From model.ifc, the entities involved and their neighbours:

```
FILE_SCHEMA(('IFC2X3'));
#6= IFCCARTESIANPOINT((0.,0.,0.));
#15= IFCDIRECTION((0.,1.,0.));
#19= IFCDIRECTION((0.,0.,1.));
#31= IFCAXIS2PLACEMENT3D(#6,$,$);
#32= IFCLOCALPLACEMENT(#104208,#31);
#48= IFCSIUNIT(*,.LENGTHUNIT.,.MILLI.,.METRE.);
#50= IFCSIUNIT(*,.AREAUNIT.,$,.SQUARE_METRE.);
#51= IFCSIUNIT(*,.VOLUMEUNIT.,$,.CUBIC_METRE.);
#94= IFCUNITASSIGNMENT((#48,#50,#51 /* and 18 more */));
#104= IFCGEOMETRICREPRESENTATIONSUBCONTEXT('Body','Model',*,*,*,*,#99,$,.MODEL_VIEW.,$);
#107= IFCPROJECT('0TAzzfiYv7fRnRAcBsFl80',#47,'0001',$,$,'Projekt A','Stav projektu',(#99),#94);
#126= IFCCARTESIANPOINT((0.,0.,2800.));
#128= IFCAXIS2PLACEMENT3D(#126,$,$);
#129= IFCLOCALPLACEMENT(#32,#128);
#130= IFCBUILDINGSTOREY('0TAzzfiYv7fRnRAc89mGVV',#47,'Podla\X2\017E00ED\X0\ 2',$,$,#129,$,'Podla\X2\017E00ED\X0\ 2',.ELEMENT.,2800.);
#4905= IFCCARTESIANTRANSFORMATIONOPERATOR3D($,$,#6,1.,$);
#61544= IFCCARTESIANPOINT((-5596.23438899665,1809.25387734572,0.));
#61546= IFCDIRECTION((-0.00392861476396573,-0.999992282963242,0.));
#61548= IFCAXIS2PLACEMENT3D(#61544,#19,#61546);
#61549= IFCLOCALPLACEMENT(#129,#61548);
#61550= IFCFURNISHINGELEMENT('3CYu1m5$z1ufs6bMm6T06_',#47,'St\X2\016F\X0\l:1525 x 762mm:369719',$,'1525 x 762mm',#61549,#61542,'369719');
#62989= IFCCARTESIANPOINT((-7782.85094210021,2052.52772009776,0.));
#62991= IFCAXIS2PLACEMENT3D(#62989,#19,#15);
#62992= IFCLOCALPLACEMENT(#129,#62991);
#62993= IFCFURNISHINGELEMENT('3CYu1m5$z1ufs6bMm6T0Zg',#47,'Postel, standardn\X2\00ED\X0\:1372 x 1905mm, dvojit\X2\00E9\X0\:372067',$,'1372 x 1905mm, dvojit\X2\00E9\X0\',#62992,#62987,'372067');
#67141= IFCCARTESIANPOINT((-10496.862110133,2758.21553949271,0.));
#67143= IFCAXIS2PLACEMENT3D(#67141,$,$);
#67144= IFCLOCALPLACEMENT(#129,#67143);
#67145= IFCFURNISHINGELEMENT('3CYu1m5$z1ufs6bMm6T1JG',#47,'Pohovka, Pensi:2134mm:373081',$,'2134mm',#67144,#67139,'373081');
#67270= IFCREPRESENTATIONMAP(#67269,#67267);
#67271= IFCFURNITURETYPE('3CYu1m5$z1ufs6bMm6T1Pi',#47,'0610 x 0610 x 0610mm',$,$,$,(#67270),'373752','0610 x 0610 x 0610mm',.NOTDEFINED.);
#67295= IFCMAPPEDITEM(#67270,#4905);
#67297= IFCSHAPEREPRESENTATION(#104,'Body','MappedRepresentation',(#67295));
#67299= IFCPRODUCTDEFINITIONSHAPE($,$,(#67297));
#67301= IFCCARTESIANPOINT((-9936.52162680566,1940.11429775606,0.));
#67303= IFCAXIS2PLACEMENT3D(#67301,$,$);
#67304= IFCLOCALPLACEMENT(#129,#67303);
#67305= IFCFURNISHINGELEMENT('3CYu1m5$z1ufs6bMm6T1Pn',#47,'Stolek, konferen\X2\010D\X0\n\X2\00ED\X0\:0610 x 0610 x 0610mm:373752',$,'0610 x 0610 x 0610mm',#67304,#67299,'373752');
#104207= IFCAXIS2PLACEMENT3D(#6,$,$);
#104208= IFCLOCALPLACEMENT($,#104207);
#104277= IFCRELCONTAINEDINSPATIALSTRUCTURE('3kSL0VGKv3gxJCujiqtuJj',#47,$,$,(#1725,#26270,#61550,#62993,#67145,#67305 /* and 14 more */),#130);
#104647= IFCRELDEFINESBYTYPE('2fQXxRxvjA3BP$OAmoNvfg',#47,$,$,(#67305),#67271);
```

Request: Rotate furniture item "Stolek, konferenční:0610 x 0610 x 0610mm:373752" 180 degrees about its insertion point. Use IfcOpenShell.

```python
import ifcopenshell
import ifcopenshell.api.geometry
import ifcopenshell.util.placement

model = ifcopenshell.open("model.ifc")

item = model.by_id(67305)
matrix = ifcopenshell.util.placement.get_local_placement(item.ObjectPlacement)
matrix = matrix @ ifcopenshell.util.placement.rotation(180, "Z")
ifcopenshell.api.geometry.edit_object_placement(model, product=item, matrix=matrix, is_si=False)

print(ifcopenshell.util.placement.get_local_placement(item.ObjectPlacement).round(3) + 0.0)

model.write("model_rev.ifc")
```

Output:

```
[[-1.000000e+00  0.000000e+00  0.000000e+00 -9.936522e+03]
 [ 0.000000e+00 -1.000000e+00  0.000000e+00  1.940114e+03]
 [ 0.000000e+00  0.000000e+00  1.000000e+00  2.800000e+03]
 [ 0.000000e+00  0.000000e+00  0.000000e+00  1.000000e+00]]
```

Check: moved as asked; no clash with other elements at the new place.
